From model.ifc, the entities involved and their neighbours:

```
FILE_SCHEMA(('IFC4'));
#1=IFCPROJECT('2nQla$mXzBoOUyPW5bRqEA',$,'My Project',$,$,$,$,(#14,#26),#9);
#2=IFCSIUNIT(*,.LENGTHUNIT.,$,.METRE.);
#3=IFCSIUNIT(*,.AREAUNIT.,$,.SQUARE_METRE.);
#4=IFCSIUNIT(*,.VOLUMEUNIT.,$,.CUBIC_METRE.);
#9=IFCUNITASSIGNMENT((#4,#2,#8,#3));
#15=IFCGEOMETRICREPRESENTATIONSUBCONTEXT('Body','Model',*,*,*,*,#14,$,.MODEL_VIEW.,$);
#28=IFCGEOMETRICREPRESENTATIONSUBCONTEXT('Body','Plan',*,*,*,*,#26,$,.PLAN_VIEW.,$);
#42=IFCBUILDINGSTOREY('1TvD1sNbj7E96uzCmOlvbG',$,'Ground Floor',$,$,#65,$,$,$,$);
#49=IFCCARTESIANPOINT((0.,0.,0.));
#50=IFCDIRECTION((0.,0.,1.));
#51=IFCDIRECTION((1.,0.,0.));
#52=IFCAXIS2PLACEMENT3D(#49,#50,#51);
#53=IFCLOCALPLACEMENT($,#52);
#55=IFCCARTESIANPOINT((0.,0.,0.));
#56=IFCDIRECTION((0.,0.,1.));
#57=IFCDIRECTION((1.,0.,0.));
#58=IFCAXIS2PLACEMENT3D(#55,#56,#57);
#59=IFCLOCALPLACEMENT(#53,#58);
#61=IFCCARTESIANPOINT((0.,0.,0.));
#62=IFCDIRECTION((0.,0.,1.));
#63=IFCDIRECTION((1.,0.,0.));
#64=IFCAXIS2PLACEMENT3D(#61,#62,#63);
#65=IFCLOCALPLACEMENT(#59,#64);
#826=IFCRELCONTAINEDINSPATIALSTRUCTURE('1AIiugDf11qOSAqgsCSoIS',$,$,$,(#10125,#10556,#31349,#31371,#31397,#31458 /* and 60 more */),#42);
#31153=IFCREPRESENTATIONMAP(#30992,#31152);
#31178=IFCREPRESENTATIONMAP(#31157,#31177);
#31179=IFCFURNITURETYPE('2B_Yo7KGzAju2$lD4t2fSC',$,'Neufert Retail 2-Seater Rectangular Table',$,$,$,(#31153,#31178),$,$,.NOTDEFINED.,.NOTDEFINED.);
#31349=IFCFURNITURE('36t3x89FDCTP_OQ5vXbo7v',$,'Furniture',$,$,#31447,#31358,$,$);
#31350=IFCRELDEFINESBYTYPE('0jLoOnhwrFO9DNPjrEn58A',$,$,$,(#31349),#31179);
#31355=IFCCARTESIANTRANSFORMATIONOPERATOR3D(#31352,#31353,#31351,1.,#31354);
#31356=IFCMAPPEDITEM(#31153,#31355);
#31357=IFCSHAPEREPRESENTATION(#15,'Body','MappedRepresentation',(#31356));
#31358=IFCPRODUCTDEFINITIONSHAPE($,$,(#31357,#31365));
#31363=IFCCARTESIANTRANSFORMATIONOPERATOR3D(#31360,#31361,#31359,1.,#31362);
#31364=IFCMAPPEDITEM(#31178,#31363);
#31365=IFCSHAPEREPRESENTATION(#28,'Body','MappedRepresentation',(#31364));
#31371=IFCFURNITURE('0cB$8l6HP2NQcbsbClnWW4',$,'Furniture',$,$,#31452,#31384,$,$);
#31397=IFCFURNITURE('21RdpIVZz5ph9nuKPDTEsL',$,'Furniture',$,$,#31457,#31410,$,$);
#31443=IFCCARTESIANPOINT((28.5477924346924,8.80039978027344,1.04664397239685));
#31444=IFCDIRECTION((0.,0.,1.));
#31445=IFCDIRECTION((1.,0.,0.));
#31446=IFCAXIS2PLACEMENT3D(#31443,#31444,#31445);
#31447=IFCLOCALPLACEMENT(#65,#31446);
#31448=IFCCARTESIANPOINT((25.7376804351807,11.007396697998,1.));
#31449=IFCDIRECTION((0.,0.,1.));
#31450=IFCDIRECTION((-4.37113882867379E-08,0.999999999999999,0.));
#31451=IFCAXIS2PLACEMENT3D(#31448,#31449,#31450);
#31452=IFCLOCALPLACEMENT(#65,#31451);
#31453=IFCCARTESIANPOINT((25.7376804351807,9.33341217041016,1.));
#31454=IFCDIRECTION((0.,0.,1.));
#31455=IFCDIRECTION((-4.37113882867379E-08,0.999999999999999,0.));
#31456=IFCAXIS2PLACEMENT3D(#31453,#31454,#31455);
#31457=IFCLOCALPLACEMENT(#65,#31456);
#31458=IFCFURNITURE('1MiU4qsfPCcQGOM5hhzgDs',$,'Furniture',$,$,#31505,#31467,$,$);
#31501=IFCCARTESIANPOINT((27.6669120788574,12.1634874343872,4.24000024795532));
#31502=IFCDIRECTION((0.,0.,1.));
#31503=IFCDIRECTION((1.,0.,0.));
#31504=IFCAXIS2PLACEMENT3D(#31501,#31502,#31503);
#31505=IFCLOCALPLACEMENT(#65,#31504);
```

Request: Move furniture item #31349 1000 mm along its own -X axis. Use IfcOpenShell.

```python
import ifcopenshell
import ifcopenshell.api.geometry
import ifcopenshell.util.placement
import ifcopenshell.util.unit

model = ifcopenshell.open("model.ifc")
unit_scale = ifcopenshell.util.unit.calculate_unit_scale(model)

item = model.by_id(31349)
matrix = ifcopenshell.util.placement.get_local_placement(item.ObjectPlacement)
matrix[:3, 3] -= matrix[:3, 0] * 1 / unit_scale
ifcopenshell.api.geometry.edit_object_placement(model, product=item, matrix=matrix, is_si=False)

print(ifcopenshell.util.placement.get_local_placement(item.ObjectPlacement).round(3) + 0.0)

model.write("model_updated.ifc")
```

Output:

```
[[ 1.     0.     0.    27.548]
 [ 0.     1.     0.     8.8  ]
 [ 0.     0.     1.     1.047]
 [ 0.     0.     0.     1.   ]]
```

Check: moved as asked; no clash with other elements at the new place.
